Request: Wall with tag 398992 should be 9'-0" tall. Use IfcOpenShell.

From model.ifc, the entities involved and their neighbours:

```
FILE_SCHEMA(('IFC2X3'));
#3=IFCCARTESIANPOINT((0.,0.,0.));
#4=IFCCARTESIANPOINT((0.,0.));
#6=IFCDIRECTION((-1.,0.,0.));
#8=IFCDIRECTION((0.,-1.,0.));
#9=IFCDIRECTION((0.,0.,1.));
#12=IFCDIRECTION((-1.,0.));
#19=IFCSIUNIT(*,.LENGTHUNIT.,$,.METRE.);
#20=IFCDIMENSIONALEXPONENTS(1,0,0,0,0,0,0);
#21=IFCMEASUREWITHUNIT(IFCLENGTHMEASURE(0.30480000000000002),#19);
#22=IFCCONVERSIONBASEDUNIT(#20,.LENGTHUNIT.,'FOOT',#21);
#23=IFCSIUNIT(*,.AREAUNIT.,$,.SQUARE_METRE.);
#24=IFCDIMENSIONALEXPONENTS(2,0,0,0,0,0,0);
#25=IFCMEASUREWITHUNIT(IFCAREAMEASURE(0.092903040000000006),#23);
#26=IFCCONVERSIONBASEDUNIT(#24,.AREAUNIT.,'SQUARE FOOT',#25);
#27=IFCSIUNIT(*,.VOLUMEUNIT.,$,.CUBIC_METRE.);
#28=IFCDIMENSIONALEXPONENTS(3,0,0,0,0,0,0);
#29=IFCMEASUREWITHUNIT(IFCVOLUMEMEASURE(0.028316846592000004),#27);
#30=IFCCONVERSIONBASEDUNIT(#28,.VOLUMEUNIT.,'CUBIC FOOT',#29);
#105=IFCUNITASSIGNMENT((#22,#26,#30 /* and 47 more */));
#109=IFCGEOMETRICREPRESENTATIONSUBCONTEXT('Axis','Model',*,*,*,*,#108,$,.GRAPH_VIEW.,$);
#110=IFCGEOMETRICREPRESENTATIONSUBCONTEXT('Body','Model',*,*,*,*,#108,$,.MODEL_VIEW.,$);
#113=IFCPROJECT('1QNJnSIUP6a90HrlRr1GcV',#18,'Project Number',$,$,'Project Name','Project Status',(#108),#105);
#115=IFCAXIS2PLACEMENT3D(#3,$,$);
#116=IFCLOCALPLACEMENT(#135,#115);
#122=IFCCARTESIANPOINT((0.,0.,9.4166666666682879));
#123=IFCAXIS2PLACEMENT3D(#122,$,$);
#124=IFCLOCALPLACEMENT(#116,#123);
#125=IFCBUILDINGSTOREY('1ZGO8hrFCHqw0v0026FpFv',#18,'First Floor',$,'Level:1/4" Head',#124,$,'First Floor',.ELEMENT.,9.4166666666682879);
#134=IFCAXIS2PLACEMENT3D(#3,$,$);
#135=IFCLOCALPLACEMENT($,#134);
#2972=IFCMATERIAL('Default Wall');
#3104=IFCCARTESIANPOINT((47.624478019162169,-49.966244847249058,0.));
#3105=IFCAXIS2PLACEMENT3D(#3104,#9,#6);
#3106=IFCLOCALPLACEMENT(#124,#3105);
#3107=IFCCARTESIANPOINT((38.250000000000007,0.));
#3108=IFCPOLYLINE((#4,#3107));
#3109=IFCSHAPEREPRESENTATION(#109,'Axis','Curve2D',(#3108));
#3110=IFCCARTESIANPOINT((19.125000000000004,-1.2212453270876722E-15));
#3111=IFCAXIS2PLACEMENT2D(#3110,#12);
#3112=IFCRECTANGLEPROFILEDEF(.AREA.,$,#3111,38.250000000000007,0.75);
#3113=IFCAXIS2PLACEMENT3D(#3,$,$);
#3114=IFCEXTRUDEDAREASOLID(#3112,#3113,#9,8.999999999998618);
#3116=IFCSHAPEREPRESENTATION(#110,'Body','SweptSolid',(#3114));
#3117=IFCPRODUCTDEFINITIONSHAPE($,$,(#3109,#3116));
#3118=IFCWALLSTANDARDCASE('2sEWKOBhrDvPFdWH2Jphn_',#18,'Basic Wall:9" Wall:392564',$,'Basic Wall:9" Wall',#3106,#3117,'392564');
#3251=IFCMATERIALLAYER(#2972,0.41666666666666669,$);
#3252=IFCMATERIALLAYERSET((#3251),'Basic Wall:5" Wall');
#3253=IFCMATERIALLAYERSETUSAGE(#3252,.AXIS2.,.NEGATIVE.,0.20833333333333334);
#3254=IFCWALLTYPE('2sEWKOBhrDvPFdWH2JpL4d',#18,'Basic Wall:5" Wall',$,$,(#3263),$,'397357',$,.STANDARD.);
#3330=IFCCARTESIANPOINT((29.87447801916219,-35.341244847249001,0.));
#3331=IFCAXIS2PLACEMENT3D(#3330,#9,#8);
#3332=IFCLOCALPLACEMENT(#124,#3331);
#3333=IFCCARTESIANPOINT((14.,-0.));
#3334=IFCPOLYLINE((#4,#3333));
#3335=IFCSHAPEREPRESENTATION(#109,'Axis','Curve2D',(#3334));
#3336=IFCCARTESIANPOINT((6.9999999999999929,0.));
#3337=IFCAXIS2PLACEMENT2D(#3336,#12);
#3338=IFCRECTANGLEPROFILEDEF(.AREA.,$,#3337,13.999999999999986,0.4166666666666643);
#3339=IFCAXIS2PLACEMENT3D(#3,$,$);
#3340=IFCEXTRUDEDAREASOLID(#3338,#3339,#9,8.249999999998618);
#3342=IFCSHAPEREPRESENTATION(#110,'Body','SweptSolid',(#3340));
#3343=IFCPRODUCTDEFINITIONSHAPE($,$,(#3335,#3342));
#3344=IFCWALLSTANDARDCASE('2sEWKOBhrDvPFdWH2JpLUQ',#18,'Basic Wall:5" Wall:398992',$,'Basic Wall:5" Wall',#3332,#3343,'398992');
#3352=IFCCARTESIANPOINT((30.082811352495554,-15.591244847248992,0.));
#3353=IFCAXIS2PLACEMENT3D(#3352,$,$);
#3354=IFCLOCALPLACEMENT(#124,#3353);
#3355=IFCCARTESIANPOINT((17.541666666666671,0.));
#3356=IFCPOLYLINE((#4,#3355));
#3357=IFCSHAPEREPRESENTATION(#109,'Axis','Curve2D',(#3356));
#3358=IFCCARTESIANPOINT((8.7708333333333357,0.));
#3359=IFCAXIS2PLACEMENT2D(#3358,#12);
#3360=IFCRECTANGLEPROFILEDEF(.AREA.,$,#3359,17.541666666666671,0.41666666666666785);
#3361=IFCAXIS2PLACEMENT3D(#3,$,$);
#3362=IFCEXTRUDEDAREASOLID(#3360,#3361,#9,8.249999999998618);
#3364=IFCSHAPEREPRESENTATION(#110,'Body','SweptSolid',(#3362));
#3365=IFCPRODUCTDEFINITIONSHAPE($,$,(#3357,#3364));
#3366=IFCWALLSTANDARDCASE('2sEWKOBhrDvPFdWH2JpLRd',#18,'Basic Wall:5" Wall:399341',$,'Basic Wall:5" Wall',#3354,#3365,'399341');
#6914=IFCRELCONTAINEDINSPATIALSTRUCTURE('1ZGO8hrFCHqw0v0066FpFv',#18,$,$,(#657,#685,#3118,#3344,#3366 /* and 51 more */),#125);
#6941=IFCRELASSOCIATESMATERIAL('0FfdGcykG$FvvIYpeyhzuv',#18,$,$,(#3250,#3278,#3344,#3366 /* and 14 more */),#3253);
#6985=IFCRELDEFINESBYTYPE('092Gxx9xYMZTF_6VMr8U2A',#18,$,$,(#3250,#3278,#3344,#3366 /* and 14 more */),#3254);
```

```python
import ifcopenshell
import ifcopenshell.geom
import ifcopenshell.util.representation
import ifcopenshell.util.shape
import ifcopenshell.util.unit

model = ifcopenshell.open("model.ifc")
unit_scale = ifcopenshell.util.unit.calculate_unit_scale(model)
settings = ifcopenshell.geom.settings()


def volume(element):
    """Net volume in cubic metres, openings subtracted."""
    shape = ifcopenshell.geom.create_shape(settings, element)
    return ifcopenshell.util.shape.get_volume(shape.geometry)


wall = model.by_guid("2sEWKOBhrDvPFdWH2JpLUQ")
before = volume(wall)

body = ifcopenshell.util.representation.get_representation(wall, "Model", "Body")
solid = body.Items[0]
old_height = solid.Depth
solid.Depth = 108 * 0.0254 / unit_scale
after = volume(wall)

print(f"height {old_height:g} -> {solid.Depth:g}, volume {before:.3f} -> {after:.3f} m3")

model.write("model_updated.ifc")
```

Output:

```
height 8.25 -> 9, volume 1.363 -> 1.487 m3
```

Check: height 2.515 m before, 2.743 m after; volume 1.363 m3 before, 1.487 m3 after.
